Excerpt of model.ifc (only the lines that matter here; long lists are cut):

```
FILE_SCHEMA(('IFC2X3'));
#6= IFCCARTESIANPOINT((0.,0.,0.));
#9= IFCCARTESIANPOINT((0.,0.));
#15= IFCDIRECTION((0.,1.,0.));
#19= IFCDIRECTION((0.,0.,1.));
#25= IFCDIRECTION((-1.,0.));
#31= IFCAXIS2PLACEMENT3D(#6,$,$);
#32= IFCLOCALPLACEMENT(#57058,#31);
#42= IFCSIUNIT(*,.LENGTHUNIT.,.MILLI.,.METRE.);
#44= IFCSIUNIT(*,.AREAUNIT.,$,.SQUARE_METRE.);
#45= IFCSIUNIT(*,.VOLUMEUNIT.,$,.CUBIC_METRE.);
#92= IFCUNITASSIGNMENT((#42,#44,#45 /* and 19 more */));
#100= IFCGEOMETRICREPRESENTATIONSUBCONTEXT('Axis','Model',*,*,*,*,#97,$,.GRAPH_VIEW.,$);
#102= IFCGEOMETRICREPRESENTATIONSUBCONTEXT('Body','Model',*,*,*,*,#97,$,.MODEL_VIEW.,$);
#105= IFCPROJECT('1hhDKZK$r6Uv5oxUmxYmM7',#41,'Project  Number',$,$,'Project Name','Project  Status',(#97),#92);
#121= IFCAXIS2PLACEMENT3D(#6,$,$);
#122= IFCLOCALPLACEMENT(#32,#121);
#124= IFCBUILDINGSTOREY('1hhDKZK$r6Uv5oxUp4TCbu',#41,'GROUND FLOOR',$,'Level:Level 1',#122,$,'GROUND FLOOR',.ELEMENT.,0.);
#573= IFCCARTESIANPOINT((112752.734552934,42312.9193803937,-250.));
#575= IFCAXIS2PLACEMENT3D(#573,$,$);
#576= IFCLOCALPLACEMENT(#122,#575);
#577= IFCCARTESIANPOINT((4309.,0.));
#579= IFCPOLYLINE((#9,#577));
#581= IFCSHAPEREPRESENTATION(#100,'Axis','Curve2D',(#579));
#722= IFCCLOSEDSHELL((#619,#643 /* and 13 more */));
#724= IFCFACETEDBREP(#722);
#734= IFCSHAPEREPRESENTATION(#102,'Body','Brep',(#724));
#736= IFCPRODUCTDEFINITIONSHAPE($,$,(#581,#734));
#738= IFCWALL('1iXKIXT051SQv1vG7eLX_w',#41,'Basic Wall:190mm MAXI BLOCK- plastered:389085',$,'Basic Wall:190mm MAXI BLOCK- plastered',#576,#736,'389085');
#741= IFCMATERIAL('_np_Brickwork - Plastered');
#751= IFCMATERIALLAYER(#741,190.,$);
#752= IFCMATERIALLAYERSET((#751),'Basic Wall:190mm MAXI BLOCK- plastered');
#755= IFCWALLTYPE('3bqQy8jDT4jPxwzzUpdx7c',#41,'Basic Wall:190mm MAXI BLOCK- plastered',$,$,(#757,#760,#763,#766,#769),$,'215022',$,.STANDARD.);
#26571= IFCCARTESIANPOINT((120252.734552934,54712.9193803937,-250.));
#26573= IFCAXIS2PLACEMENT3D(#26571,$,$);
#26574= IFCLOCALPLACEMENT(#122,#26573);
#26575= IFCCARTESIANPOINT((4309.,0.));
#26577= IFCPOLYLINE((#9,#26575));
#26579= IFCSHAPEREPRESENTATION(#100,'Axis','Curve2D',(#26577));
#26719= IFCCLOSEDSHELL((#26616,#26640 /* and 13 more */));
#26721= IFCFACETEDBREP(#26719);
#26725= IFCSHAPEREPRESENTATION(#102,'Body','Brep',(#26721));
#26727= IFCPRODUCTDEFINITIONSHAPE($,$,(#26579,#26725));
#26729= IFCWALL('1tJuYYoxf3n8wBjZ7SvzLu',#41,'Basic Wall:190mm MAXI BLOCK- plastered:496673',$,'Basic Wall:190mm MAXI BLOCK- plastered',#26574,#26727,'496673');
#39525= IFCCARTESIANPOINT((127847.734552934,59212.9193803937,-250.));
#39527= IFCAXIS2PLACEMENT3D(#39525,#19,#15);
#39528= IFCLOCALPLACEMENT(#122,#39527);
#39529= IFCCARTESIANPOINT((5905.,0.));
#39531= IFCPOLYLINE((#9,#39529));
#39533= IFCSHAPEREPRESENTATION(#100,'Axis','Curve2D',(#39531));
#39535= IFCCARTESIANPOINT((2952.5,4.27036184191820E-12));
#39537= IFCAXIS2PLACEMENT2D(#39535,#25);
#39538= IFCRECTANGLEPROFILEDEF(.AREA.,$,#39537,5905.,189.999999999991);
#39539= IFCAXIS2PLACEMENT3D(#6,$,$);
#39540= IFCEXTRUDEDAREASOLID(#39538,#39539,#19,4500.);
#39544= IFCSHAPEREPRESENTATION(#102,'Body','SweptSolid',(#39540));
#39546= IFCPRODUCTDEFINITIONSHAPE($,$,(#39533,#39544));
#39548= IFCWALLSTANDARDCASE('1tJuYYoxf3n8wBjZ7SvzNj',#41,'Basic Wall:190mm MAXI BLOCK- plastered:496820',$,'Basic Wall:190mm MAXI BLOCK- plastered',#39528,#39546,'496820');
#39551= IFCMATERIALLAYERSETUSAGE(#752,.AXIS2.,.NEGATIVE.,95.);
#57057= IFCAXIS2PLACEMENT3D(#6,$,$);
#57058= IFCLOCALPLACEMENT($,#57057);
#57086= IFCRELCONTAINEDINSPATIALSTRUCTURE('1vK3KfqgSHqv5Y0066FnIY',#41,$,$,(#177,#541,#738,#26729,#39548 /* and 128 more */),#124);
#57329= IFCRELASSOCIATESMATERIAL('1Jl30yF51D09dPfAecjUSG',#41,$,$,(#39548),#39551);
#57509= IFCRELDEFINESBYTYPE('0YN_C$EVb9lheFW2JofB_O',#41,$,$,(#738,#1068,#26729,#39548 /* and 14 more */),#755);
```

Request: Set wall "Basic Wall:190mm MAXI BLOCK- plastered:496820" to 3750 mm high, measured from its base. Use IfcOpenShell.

```python
import ifcopenshell
import ifcopenshell.geom
import ifcopenshell.util.representation
import ifcopenshell.util.shape

model = ifcopenshell.open("model.ifc")
settings = ifcopenshell.geom.settings()


def volume(element):
    """Net volume in cubic metres, openings subtracted."""
    shape = ifcopenshell.geom.create_shape(settings, element)
    return ifcopenshell.util.shape.get_volume(shape.geometry)


wall = model.by_guid("1tJuYYoxf3n8wBjZ7SvzNj")
before = volume(wall)

body = ifcopenshell.util.representation.get_representation(wall, "Model", "Body")
solid = body.Items[0]
old_height = solid.Depth
solid.Depth = 3750.0
after = volume(wall)

print(f"height {old_height:g} -> {solid.Depth:g}, volume {before:.3f} -> {after:.3f} m3")

model.write("model_edited.ifc")
```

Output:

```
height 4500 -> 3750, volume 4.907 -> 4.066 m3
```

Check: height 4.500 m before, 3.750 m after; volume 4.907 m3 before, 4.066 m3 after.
